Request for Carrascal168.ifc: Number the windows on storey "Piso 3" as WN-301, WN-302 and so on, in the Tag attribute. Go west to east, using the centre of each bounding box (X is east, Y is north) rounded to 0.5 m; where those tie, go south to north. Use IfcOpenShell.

First a look at what the model holds.

```python
import ifcopenshell
import ifcopenshell.util.element
import ifcopenshell.util.placement

model = ifcopenshell.open("Carrascal168.ifc")
print(model.schema)
storey = next(s for s in model.by_type("IfcBuildingStorey") if s.Name == "Piso 3")
windows = [e for e in ifcopenshell.util.element.get_decomposition(storey) if e.is_a("IfcWindow")]
for e in sorted(windows, key=lambda e: e.id()):
    origin = ifcopenshell.util.placement.get_local_placement(e.ObjectPlacement)[:3, 3]
    print(e.id(), e.Tag, e.Name, origin.round(2) + 0.0, sep=" | ")
```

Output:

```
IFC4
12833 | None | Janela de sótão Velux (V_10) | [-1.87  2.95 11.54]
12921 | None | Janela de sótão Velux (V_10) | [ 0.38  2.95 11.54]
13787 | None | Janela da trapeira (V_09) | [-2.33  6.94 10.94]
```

```python
import ifcopenshell
import ifcopenshell.geom
import ifcopenshell.util.element
import ifcopenshell.util.shape

model = ifcopenshell.open("Carrascal168.ifc")
settings = ifcopenshell.geom.settings()
settings.set("use-world-coords", True)


def centre(element):
    shape = ifcopenshell.geom.create_shape(settings, element)
    return ifcopenshell.util.shape.get_bbox_centroid(shape.geometry)


storey = next(s for s in model.by_type("IfcBuildingStorey") if s.Name == "Piso 3")
windows = [e for e in ifcopenshell.util.element.get_decomposition(storey) if e.is_a("IfcWindow")]

# Insertion points can sit at a corner or the storey origin, so sort by the geometry (in metres).
centres = {e: centre(e) for e in windows}
windows.sort(key=lambda e: (round(centres[e][0] / 0.5), centres[e][1]))

for i, e in enumerate(windows, start=1):
    number = f"WN-3{i:02d}"
    e.Tag = number
    print(e.id(), number)

model.write("Carrascal168_v2.ifc")
```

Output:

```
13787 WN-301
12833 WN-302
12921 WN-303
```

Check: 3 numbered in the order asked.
